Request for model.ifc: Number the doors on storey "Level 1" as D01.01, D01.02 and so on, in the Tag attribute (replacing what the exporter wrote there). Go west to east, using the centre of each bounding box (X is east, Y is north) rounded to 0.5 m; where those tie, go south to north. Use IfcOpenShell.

First a look at what the model holds.

```python
import ifcopenshell
import ifcopenshell.util.element
import ifcopenshell.util.placement

model = ifcopenshell.open("model.ifc")
print(model.schema)
storey = next(s for s in model.by_type("IfcBuildingStorey") if s.Name == "Level 1")
doors = [e for e in ifcopenshell.util.element.get_decomposition(storey) if e.is_a("IfcDoor")]
for e in sorted(doors, key=lambda e: e.id()):
    origin = ifcopenshell.util.placement.get_local_placement(e.ObjectPlacement)[:3, 3]
    print(e.id(), e.Tag, e.Name, origin.round(2) + 0.0, sep=" | ")
```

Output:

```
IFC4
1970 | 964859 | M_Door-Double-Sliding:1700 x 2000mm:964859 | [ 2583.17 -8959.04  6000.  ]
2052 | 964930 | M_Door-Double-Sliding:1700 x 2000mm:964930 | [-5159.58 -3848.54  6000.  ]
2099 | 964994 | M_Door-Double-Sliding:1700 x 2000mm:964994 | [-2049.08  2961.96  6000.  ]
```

```python
import ifcopenshell
import ifcopenshell.geom
import ifcopenshell.util.element
import ifcopenshell.util.shape

model = ifcopenshell.open("model.ifc")
settings = ifcopenshell.geom.settings()
settings.set("use-world-coords", True)


def centre(element):
    shape = ifcopenshell.geom.create_shape(settings, element)
    return ifcopenshell.util.shape.get_bbox_centroid(shape.geometry)


storey = next(s for s in model.by_type("IfcBuildingStorey") if s.Name == "Level 1")
doors = [e for e in ifcopenshell.util.element.get_decomposition(storey) if e.is_a("IfcDoor")]

# Insertion points can sit at a corner or the storey origin, so sort by the geometry (in metres).
centres = {e: centre(e) for e in doors}
doors.sort(key=lambda e: (round(centres[e][0] / 0.5), centres[e][1]))

for i, e in enumerate(doors, start=1):
    number = f"D01.{i:02d}"
    e.Tag = number
    print(e.id(), number)

model.write("model_edited.ifc")
```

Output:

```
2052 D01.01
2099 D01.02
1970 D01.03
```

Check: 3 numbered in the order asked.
